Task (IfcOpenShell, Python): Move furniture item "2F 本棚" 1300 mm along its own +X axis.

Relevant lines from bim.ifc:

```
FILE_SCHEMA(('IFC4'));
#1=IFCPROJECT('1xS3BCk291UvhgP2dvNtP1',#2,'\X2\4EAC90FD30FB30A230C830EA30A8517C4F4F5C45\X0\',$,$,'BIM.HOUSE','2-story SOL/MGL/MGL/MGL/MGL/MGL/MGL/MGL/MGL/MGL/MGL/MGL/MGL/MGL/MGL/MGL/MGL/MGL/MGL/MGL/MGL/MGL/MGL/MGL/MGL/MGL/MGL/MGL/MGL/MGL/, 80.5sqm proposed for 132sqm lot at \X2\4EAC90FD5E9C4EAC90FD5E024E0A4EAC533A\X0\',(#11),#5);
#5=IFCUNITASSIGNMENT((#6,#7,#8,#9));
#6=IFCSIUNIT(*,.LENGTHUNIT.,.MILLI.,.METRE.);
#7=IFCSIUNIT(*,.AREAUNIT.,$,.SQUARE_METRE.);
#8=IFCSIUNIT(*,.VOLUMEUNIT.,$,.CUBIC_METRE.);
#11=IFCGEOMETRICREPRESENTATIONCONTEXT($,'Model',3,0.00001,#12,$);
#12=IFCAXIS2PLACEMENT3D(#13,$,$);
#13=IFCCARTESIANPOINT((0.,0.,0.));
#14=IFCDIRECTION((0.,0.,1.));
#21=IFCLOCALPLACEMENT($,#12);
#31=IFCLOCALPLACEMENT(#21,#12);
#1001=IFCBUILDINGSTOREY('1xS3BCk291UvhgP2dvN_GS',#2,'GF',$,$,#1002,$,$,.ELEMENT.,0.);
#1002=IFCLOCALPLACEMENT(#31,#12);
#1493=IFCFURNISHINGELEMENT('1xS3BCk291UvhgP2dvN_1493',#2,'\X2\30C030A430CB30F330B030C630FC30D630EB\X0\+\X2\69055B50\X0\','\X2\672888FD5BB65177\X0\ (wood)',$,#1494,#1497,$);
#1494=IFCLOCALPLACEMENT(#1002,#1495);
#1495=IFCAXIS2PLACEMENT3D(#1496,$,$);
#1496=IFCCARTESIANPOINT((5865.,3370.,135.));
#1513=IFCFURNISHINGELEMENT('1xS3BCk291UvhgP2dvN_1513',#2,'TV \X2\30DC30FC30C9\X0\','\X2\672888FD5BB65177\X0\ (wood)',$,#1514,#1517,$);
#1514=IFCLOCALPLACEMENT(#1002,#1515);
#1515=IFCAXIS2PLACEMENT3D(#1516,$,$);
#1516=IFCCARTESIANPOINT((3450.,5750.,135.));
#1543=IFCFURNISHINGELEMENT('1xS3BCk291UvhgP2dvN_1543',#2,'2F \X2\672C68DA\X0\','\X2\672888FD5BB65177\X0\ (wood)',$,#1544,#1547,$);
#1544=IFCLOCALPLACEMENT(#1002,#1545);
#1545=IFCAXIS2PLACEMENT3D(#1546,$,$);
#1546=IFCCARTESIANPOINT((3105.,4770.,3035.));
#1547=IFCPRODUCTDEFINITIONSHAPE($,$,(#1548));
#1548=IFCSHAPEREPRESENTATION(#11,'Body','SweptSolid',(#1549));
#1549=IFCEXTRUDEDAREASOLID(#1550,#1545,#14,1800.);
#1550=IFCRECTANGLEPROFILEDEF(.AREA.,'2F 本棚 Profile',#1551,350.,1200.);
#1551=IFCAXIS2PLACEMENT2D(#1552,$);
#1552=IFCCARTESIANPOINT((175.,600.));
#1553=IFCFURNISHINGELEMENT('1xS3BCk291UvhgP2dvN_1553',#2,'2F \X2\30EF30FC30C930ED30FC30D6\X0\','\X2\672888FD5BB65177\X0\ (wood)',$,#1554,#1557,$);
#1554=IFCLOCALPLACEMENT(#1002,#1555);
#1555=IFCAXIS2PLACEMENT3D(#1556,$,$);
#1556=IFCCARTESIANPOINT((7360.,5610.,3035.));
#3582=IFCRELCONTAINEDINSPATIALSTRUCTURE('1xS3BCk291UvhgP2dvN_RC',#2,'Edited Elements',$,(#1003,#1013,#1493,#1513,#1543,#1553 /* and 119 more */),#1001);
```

```python
import ifcopenshell
import ifcopenshell.api.geometry
import ifcopenshell.util.placement

model = ifcopenshell.open("bim.ifc")

item = model.by_guid("1xS3BCk291UvhgP2dvN_1543")
matrix = ifcopenshell.util.placement.get_local_placement(item.ObjectPlacement)
matrix[:3, 3] += matrix[:3, 0] * 1300.0
ifcopenshell.api.geometry.edit_object_placement(model, product=item, matrix=matrix, is_si=False)

print(ifcopenshell.util.placement.get_local_placement(item.ObjectPlacement).round(3) + 0.0)

model.write("bim_rev.ifc")
```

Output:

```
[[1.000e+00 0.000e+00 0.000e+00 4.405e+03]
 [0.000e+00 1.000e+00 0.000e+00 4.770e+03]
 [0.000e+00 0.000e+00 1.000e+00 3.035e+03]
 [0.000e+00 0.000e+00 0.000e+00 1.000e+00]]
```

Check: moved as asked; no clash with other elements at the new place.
